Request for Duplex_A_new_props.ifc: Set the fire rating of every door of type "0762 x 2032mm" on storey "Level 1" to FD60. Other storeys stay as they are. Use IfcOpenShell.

First a look at what the model holds.

```python
import ifcopenshell
import ifcopenshell.util.element

model = ifcopenshell.open("Duplex_A_new_props.ifc")
print(model.schema)
storey = next(s for s in model.by_type("IfcBuildingStorey") if s.Name == "Level 1")
doors = [e for e in ifcopenshell.util.element.get_decomposition(storey) if e.is_a("IfcDoor")]
seen = {}
for e in doors:
    element_type = ifcopenshell.util.element.get_type(e)
    key = (element_type.Name if element_type != e and element_type else None, ifcopenshell.util.element.get_pset(e, "Pset_DoorCommon", "FireRating"))
    seen[key] = seen.get(key, 0) + 1
for (name, value), count in sorted(seen.items(), key=str):
    print(count, "x", name, "|", value)
```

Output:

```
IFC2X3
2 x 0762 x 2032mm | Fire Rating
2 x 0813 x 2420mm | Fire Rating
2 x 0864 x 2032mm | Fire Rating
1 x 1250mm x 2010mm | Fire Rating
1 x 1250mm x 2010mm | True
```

```python
import ifcopenshell
import ifcopenshell.api.pset
import ifcopenshell.util.element

model = ifcopenshell.open("Duplex_A_new_props.ifc")

storey = next(s for s in model.by_type("IfcBuildingStorey") if s.Name == "Level 1")
doors = [e for e in ifcopenshell.util.element.get_decomposition(storey) if e.is_a("IfcDoor")]

count = 0
for e in doors:
    element_type = ifcopenshell.util.element.get_type(e)
    if element_type in (None, e) or element_type.Name != "0762 x 2032mm":
        continue
    # add_pset returns the element's existing set when there is one.
    pset = ifcopenshell.api.pset.add_pset(model, product=e, name="Pset_DoorCommon")
    ifcopenshell.api.pset.edit_pset(model, pset=pset, properties={"FireRating": "FD60"})
    count += 1

print(count, "doors updated")

model.write("Duplex_A_new_props_updated.ifc")
```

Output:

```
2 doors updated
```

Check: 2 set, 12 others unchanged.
